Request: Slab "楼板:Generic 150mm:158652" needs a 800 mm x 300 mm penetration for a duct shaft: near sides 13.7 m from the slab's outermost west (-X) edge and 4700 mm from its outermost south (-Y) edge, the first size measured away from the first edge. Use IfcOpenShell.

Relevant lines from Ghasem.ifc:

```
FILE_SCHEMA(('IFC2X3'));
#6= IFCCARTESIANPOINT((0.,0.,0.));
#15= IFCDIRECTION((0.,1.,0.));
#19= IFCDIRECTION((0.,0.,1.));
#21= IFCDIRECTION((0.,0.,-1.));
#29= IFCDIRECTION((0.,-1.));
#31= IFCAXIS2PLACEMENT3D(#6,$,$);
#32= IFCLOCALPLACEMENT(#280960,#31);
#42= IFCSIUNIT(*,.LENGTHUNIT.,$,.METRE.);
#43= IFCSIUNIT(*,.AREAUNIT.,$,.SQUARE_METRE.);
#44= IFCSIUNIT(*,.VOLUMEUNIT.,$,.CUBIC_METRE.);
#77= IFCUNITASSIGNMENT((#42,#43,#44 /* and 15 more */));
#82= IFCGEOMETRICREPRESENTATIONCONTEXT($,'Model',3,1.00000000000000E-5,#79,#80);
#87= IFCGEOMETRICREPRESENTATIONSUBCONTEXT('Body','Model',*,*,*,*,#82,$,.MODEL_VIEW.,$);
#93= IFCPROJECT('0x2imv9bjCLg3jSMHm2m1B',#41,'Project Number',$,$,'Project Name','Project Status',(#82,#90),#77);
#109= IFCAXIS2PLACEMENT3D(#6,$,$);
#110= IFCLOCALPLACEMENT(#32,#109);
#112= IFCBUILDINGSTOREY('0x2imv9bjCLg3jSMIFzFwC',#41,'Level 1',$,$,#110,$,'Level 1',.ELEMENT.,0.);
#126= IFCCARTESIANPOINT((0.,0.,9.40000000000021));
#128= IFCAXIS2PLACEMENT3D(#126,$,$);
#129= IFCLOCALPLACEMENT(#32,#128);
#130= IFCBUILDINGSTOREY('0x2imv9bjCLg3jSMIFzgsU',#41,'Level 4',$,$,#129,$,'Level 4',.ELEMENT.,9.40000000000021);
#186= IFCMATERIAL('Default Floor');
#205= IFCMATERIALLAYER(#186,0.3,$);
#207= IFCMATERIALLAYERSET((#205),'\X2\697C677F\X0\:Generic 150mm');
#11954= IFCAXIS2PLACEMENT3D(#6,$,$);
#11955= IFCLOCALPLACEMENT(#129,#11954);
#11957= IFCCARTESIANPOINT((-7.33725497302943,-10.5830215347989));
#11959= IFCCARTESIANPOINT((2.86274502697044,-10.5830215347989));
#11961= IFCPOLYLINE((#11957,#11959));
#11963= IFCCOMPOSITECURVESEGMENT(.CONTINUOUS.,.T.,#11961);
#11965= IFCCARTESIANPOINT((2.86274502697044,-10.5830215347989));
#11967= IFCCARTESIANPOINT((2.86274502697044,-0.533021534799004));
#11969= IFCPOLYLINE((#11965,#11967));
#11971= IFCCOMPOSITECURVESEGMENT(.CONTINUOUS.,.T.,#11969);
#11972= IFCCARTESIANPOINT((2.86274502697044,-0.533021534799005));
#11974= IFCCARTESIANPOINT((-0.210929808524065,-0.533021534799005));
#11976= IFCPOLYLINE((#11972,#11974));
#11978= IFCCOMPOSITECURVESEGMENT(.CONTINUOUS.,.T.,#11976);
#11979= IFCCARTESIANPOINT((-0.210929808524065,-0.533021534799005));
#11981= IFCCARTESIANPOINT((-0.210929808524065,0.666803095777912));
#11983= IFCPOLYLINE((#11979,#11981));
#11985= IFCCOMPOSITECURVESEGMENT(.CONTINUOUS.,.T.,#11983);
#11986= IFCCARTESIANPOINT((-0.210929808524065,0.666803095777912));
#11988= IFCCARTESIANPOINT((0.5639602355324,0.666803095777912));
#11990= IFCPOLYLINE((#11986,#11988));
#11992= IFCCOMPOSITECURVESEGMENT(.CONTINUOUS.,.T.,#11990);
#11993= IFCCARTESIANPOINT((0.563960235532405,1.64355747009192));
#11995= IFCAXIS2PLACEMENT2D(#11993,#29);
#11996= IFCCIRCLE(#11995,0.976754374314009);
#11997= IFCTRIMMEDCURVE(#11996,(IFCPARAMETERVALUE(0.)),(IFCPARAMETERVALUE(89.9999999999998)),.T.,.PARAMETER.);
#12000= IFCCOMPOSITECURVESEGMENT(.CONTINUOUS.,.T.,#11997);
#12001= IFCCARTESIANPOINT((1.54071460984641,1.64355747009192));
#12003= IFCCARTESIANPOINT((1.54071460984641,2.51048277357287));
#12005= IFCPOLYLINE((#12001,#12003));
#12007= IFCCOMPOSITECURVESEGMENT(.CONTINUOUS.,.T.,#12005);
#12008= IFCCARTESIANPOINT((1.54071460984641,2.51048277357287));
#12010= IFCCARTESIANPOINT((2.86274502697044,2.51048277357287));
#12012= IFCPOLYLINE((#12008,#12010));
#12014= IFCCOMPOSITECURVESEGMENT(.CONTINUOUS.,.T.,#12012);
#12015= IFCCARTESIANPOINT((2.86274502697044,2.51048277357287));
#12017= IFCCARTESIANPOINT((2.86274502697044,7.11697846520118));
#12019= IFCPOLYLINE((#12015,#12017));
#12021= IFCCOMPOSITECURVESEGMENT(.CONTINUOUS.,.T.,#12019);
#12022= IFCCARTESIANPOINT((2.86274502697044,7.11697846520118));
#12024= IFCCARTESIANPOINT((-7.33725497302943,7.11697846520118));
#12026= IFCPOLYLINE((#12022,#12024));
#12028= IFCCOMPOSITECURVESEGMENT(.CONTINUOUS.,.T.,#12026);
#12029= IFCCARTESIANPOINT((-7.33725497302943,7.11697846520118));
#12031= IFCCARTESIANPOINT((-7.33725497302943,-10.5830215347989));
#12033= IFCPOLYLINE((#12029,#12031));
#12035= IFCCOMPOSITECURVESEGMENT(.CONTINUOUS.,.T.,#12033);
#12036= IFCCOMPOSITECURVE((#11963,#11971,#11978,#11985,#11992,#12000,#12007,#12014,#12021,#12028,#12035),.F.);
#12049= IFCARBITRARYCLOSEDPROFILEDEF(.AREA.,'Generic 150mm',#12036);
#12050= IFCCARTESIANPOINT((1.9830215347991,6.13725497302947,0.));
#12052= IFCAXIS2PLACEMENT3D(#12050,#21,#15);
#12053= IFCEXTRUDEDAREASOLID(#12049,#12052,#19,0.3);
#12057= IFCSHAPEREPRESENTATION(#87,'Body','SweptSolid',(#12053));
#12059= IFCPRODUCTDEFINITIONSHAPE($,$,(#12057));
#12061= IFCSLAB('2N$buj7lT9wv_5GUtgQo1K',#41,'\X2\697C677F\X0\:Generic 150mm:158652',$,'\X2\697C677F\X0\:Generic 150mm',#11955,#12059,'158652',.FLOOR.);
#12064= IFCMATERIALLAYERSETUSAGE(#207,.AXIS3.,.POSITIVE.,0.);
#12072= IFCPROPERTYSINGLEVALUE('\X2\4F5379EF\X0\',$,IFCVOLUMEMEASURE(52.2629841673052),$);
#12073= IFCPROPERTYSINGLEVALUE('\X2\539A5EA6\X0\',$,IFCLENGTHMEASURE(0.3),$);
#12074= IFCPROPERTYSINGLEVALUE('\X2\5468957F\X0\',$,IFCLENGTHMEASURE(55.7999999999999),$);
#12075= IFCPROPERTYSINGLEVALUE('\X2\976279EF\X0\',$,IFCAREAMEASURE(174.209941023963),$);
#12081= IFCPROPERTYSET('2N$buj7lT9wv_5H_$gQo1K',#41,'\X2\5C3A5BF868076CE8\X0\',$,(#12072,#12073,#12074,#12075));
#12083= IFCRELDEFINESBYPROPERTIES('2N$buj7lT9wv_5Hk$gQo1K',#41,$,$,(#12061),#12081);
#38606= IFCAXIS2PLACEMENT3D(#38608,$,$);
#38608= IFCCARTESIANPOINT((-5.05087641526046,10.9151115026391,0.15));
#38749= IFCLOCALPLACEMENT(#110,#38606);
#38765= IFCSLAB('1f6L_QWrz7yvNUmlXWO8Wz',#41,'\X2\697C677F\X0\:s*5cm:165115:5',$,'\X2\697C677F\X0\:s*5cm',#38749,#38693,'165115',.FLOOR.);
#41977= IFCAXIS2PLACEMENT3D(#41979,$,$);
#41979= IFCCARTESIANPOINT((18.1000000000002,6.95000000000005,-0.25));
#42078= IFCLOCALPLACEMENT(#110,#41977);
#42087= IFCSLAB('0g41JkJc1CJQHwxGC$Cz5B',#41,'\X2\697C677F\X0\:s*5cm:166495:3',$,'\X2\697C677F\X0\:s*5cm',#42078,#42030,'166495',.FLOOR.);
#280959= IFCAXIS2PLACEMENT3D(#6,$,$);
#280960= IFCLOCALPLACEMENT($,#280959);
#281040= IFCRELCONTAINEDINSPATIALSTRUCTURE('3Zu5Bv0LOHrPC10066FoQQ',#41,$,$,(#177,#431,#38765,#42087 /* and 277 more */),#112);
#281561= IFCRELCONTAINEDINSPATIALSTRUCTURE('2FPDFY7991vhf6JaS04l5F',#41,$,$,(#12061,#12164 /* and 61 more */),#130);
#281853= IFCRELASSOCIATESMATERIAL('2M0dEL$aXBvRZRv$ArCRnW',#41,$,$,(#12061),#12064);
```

```python
import numpy as np
import ifcopenshell
import ifcopenshell.api.feature
import ifcopenshell.api.geometry
import ifcopenshell.api.pset
import ifcopenshell.api.root
import ifcopenshell.geom
import ifcopenshell.util.element
import ifcopenshell.util.placement
import ifcopenshell.util.representation
import ifcopenshell.util.shape
import ifcopenshell.util.unit

model = ifcopenshell.open("Ghasem.ifc")
unit_scale = ifcopenshell.util.unit.calculate_unit_scale(model)
area_scale = ifcopenshell.util.unit.calculate_unit_scale(model, "AREAUNIT")
volume_scale = ifcopenshell.util.unit.calculate_unit_scale(model, "VOLUMEUNIT")
settings = ifcopenshell.geom.settings()


def volume(element):
    """Net volume in cubic metres, openings subtracted."""
    shape = ifcopenshell.geom.create_shape(settings, element)
    return ifcopenshell.util.shape.get_volume(shape.geometry)


slab = model.by_guid("2N$buj7lT9wv_5GUtgQo1K")
before = volume(slab)

# Extent in the slab's own axes, in metres. The edges named are its -X and -Y sides.
slab_shape = ifcopenshell.geom.create_shape(settings, slab)
vertices = ifcopenshell.util.shape.get_vertices(slab_shape.geometry)
x_min, y_min, bottom = vertices.min(axis=0)
top = vertices[:, 2].max()

opening = ifcopenshell.api.root.create_entity(model, ifc_class="IfcOpeningElement", name="Duct shaft opening")
context = ifcopenshell.util.representation.get_context(model, "Model", "Body", "MODEL_VIEW")
width, depth = 0.8, 0.3
outline = [(0.0, 0.0), (width, 0.0), (width, depth), (0.0, depth), (0.0, 0.0)]
# Overshoot both faces by 50 mm so the cut is clean.
shape = ifcopenshell.api.geometry.add_slab_representation(
    model, context=context, depth=top - bottom + 0.1, polyline=outline
)
ifcopenshell.api.geometry.assign_representation(model, product=opening, representation=shape)

matrix = ifcopenshell.util.placement.get_local_placement(slab.ObjectPlacement)
matrix[:, 3] = matrix @ np.append(np.array([x_min + 13.7, y_min + 4.7, bottom - 0.05]) / unit_scale, 1.0)
ifcopenshell.api.geometry.edit_object_placement(model, product=opening, matrix=matrix, is_si=False)
ifcopenshell.api.feature.add_feature(model, feature=opening, element=slab)

after = volume(slab)

# Update the slab's stored quantities.
pset = model.by_id(ifcopenshell.util.element.get_pset(slab, "尺寸标注", should_inherit=False)["id"])
ifcopenshell.api.pset.edit_pset(model, pset=pset, properties={
    "体积": model.create_entity("IfcVolumeMeasure", after / volume_scale),
    "面积": model.create_entity("IfcAreaMeasure", after / (top - bottom) / area_scale),
})

print(f"slab volume {before:.3f} -> {after:.3f} m3")

model.write("Ghasem_rev.ifc")
```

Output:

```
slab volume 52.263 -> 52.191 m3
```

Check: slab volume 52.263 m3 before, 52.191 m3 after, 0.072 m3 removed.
